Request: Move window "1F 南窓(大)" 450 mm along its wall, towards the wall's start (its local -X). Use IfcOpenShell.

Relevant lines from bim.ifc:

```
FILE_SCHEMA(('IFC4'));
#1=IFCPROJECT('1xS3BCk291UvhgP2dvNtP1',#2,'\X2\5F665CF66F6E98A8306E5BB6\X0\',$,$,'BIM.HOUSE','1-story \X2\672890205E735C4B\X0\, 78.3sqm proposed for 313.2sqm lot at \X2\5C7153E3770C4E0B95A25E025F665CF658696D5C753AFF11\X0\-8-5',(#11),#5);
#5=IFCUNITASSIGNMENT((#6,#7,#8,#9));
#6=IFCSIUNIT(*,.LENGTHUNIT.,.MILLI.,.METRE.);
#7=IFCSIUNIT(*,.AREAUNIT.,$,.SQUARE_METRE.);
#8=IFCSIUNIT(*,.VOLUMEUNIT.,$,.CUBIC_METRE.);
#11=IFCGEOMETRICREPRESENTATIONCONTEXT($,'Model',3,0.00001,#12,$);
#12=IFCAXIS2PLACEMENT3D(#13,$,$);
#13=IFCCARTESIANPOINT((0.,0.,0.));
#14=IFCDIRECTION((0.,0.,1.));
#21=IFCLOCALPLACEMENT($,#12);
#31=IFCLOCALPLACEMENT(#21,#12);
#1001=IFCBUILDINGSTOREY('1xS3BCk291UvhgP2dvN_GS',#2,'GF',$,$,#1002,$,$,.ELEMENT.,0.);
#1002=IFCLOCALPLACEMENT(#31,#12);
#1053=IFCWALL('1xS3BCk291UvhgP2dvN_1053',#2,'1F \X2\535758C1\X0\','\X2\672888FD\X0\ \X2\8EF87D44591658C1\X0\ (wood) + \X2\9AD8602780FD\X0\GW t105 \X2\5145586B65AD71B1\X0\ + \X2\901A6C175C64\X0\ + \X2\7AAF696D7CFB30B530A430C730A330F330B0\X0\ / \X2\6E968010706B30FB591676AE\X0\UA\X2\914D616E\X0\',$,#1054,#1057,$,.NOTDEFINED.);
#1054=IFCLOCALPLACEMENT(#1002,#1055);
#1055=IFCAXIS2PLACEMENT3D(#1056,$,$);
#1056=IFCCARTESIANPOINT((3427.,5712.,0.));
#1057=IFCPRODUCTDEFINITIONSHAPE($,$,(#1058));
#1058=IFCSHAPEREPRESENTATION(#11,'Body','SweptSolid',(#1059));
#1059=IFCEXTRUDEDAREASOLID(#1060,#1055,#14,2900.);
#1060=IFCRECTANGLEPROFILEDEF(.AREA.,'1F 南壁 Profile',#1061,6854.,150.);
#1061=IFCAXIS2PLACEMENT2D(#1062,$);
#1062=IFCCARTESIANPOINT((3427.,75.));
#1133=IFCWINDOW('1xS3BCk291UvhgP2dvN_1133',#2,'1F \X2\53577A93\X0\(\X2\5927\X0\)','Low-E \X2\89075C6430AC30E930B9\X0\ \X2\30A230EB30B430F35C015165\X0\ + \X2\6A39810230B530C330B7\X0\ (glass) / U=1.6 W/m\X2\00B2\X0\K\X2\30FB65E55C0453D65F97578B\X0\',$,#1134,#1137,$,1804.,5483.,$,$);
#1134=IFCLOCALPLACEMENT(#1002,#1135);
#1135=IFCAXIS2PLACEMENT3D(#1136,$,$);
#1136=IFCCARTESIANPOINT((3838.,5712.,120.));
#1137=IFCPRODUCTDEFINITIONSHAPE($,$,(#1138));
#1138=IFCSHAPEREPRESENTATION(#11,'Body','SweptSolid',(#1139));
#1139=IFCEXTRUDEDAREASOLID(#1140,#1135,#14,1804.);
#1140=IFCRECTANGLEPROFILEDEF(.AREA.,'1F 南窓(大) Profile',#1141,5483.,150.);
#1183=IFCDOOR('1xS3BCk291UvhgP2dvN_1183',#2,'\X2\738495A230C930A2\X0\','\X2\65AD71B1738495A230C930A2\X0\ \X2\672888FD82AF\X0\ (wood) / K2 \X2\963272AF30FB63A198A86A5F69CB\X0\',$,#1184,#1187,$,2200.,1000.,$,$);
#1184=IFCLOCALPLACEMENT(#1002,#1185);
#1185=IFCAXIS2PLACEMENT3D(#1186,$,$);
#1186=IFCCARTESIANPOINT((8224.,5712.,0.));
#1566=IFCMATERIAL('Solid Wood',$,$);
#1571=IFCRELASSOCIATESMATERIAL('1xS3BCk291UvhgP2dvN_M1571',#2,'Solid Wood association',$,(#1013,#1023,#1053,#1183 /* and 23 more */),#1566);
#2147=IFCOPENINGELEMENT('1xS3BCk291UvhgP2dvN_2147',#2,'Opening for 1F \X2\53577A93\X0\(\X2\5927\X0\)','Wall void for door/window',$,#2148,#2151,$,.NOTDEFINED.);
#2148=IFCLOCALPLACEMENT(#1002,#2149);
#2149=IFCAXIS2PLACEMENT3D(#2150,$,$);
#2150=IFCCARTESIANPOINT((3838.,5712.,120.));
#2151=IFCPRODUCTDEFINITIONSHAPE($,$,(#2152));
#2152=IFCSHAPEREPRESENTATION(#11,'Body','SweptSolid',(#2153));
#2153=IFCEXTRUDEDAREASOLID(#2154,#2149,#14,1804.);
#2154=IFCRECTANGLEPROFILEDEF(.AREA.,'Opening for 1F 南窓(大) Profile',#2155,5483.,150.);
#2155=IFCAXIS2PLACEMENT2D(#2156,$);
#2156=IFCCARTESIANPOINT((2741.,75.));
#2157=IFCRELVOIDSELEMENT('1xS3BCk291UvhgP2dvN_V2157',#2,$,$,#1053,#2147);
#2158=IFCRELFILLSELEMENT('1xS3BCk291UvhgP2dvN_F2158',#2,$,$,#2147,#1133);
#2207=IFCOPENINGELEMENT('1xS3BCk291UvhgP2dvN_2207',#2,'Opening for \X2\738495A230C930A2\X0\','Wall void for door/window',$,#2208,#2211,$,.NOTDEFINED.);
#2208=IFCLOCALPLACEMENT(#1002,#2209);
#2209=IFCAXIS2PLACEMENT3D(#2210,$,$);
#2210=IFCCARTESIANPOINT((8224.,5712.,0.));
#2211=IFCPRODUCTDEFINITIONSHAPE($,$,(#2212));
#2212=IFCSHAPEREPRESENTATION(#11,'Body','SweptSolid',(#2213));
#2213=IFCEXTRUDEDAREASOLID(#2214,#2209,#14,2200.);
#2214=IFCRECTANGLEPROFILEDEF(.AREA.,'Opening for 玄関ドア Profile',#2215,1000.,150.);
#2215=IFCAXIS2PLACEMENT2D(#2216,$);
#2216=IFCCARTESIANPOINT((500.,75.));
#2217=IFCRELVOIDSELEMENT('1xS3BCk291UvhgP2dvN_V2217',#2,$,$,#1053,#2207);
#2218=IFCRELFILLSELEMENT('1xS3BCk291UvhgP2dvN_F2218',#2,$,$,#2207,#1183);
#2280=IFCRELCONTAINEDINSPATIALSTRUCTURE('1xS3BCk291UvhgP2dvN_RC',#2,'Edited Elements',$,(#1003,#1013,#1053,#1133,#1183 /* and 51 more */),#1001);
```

```python
import ifcopenshell
import ifcopenshell.api.geometry
import ifcopenshell.util.placement
import ifcopenshell.util.unit

model = ifcopenshell.open("bim.ifc")
unit_scale = ifcopenshell.util.unit.calculate_unit_scale(model)

window = model.by_guid("1xS3BCk291UvhgP2dvN_1133")
opening = window.FillsVoids[0].RelatingOpeningElement
wall = opening.VoidsElements[0].RelatingBuildingElement

wall_matrix = ifcopenshell.util.placement.get_local_placement(wall.ObjectPlacement)
shift = wall_matrix[:3, 0] * -0.45 / unit_scale
before = ifcopenshell.util.placement.get_local_placement(window.ObjectPlacement)[:3, 3].copy()

# The window is not placed relative to its opening, so move both.
for product in (opening, window):
    matrix = ifcopenshell.util.placement.get_local_placement(product.ObjectPlacement)
    matrix[:3, 3] += shift
    ifcopenshell.api.geometry.edit_object_placement(model, product=product, matrix=matrix, is_si=False)

after = ifcopenshell.util.placement.get_local_placement(window.ObjectPlacement)[:3, 3]
print("window moved by", (after - before).round(3) + 0.0)

model.write("bim_v2.ifc")
```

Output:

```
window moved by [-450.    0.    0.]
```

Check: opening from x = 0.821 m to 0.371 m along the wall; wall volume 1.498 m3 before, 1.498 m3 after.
